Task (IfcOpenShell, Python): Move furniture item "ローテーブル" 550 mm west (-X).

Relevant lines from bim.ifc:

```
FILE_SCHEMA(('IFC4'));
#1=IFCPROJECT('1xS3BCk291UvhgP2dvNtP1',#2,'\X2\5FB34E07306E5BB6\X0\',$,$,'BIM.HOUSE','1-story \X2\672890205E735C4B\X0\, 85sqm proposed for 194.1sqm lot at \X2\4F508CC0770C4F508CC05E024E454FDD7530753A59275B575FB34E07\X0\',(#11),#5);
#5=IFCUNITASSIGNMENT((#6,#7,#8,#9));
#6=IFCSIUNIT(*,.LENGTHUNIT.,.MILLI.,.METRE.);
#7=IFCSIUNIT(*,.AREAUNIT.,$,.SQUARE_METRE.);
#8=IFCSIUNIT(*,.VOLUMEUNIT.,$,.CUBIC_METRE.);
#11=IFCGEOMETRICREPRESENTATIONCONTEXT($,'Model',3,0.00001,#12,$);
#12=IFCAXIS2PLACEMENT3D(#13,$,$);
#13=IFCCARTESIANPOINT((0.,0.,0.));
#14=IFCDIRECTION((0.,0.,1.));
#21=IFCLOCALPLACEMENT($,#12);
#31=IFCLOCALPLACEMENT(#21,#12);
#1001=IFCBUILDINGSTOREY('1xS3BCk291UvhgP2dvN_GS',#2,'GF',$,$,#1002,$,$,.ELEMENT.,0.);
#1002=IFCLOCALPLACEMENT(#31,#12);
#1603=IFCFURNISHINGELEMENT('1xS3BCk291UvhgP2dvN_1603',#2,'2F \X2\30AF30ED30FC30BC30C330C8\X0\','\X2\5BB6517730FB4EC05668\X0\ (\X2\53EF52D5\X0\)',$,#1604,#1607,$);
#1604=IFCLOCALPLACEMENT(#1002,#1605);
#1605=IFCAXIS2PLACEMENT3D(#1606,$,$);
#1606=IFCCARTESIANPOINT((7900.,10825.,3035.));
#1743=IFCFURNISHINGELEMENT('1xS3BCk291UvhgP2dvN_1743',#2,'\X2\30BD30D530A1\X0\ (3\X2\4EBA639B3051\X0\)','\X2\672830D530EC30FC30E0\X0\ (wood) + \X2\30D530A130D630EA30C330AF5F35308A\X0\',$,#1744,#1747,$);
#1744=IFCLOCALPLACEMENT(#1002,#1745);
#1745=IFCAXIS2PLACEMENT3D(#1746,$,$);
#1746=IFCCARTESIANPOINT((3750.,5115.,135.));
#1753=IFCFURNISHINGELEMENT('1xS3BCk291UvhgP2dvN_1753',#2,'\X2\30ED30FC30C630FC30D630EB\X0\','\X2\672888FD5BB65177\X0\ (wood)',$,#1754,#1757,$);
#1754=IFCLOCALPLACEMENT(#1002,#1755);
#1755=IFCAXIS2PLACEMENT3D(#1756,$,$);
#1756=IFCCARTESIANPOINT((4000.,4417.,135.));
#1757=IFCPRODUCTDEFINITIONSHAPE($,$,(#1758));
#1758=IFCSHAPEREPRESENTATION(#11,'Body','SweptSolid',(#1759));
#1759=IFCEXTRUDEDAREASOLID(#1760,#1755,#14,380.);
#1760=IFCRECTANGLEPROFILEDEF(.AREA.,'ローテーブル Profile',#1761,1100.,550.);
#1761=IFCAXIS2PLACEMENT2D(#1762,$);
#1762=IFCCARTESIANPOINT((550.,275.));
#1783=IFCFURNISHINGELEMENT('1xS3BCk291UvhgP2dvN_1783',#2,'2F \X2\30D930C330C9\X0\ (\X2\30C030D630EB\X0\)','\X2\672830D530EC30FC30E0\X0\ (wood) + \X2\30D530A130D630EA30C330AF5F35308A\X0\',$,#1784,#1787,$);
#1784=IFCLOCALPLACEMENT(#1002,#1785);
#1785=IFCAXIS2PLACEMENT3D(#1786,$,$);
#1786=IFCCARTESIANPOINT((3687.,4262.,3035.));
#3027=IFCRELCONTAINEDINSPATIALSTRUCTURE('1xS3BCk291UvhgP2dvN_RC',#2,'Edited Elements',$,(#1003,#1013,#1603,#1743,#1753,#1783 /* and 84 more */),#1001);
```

```python
import ifcopenshell
import ifcopenshell.api.geometry
import ifcopenshell.util.placement

model = ifcopenshell.open("bim.ifc")

item = model.by_guid("1xS3BCk291UvhgP2dvN_1753")
matrix = ifcopenshell.util.placement.get_local_placement(item.ObjectPlacement)
matrix[0, 3] -= 550.0
ifcopenshell.api.geometry.edit_object_placement(model, product=item, matrix=matrix, is_si=False)

print(ifcopenshell.util.placement.get_local_placement(item.ObjectPlacement).round(3) + 0.0)

model.write("bim_updated.ifc")
```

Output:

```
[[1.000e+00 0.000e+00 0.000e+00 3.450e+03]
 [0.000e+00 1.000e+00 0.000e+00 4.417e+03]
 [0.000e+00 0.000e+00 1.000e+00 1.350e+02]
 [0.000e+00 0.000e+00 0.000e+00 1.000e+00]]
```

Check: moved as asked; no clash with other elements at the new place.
